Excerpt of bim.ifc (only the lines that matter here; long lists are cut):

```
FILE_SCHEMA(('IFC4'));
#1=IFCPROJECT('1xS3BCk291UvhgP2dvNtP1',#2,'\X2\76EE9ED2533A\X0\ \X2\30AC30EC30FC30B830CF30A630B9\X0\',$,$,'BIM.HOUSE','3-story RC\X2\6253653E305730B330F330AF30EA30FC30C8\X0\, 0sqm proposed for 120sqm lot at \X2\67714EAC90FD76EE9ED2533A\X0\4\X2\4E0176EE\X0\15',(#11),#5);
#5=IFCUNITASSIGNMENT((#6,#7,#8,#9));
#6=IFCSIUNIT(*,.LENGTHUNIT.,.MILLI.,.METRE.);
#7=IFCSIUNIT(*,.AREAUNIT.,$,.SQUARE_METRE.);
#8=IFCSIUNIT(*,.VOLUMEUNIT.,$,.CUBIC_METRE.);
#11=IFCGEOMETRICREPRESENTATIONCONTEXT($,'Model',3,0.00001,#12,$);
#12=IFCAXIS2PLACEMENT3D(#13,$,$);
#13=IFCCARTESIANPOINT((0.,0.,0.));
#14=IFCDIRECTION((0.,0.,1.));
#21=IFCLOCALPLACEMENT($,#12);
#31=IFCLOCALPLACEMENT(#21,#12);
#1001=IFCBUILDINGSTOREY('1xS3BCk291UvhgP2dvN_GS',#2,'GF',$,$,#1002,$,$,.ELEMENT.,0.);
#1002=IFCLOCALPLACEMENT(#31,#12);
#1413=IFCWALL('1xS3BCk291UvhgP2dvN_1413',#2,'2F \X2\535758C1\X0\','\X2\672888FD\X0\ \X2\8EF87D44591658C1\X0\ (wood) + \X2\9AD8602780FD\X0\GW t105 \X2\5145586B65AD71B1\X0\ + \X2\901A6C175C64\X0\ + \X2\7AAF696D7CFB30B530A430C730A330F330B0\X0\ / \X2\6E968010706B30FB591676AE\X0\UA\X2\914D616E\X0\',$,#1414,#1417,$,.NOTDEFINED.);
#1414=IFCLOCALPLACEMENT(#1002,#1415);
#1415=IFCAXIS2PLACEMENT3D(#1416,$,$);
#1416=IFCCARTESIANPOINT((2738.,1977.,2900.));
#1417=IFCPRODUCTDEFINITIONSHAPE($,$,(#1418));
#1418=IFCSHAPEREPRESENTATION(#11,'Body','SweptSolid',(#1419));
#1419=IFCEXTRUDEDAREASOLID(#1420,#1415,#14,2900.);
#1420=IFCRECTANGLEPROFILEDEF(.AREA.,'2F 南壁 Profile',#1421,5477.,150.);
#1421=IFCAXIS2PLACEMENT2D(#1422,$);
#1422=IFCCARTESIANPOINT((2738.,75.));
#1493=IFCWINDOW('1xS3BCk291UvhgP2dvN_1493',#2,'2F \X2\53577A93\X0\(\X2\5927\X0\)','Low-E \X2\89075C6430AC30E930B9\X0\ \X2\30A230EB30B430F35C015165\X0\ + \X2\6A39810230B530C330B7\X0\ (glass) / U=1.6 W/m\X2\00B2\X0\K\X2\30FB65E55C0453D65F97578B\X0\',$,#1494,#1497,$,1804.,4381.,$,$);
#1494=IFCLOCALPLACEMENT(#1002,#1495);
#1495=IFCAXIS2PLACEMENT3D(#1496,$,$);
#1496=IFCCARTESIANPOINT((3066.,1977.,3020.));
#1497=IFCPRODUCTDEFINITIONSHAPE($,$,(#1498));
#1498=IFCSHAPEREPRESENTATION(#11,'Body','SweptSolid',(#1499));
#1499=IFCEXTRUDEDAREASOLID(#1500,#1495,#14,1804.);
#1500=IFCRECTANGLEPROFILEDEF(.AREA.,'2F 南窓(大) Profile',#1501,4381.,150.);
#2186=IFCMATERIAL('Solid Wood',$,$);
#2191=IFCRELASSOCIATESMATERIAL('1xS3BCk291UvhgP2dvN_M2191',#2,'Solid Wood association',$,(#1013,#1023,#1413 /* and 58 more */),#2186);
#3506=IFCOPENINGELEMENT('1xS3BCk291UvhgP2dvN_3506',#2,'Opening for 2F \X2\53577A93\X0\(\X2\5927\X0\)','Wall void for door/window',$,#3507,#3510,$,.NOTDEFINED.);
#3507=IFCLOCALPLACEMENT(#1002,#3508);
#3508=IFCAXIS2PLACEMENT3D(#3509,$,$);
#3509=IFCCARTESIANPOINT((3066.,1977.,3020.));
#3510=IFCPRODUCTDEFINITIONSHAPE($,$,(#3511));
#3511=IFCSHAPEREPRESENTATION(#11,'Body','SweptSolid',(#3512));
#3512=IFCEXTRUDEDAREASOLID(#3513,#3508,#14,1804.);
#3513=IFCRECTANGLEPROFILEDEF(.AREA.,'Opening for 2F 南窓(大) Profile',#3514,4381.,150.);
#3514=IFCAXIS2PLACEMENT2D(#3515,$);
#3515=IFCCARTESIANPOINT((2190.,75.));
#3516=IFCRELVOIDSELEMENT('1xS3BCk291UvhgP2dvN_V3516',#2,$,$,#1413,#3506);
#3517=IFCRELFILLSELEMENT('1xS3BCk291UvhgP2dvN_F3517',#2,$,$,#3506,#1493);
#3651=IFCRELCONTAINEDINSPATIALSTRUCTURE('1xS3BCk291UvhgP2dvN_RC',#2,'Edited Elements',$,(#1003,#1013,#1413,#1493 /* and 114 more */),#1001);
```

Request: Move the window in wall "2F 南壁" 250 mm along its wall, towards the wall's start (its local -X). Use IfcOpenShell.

```python
import ifcopenshell
import ifcopenshell.api.geometry
import ifcopenshell.util.placement
import ifcopenshell.util.unit

model = ifcopenshell.open("bim.ifc")
unit_scale = ifcopenshell.util.unit.calculate_unit_scale(model)

window = model.by_guid("1xS3BCk291UvhgP2dvN_1493")
opening = window.FillsVoids[0].RelatingOpeningElement
wall = opening.VoidsElements[0].RelatingBuildingElement

wall_matrix = ifcopenshell.util.placement.get_local_placement(wall.ObjectPlacement)
shift = wall_matrix[:3, 0] * -0.25 / unit_scale
before = ifcopenshell.util.placement.get_local_placement(window.ObjectPlacement)[:3, 3].copy()

# The window is not placed relative to its opening, so move both.
for product in (opening, window):
    matrix = ifcopenshell.util.placement.get_local_placement(product.ObjectPlacement)
    matrix[:3, 3] += shift
    ifcopenshell.api.geometry.edit_object_placement(model, product=product, matrix=matrix, is_si=False)

after = ifcopenshell.util.placement.get_local_placement(window.ObjectPlacement)[:3, 3]
print("window moved by", (after - before).round(3) + 0.0)

model.write("bim-out.ifc")
```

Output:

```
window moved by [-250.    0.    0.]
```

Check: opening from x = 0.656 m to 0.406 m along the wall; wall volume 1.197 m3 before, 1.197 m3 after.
